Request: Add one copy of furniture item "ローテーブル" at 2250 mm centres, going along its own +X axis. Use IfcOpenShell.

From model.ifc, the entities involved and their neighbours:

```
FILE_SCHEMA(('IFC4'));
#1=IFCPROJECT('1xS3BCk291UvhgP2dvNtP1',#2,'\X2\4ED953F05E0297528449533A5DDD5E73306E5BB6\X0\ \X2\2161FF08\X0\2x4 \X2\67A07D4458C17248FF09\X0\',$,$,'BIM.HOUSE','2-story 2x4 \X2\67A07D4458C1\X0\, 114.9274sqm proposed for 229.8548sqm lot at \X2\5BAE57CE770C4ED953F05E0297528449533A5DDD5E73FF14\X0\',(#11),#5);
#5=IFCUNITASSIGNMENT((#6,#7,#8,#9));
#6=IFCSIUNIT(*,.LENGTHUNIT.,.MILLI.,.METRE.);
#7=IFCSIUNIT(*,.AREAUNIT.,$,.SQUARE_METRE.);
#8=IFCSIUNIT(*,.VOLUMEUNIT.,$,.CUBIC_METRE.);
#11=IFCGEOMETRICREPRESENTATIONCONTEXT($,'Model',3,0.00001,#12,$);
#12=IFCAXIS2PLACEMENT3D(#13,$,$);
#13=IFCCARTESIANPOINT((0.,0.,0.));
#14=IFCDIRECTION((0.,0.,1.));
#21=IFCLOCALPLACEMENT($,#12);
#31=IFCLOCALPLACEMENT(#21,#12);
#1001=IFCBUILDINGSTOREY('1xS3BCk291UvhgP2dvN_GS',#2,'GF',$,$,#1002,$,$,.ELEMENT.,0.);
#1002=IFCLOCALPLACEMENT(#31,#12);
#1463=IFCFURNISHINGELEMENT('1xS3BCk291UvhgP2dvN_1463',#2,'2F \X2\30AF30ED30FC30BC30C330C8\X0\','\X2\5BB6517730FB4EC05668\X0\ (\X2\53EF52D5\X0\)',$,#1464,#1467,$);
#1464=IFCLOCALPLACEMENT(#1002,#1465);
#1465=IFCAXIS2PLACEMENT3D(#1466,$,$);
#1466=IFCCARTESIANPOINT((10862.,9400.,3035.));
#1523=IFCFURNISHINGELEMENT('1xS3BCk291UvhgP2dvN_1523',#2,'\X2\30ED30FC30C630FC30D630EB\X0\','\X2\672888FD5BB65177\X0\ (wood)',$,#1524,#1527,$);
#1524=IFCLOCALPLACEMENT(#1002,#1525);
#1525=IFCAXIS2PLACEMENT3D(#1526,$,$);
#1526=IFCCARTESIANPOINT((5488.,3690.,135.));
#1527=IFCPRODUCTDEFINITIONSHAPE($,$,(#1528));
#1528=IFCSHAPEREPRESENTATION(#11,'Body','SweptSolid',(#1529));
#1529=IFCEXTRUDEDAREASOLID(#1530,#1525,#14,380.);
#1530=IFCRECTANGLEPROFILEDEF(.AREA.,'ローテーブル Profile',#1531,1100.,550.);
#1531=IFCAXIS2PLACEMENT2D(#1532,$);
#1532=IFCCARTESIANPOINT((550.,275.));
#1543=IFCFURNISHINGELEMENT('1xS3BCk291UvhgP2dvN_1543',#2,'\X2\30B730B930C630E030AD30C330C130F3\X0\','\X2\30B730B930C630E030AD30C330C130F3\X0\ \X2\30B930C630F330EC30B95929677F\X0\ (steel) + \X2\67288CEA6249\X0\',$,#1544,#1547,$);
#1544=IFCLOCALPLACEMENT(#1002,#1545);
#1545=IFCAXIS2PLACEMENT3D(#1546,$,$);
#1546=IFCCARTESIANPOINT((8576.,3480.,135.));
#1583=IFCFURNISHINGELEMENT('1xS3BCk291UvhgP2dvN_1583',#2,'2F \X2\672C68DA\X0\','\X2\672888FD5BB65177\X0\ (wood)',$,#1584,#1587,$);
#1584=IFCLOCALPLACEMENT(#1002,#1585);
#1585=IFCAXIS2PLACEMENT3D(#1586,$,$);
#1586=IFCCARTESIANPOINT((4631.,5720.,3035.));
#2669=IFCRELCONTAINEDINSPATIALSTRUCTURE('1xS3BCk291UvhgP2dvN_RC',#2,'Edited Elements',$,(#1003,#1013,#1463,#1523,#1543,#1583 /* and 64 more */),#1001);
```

```python
import ifcopenshell
import ifcopenshell.api.geometry
import ifcopenshell.api.root
import ifcopenshell.util.element
import ifcopenshell.util.placement

model = ifcopenshell.open("model.ifc")


def reuse_history(source, copy):
    """copy_class also copies each property set's owner history, people and application; keep the originals."""
    for rel in copy.IsDefinedBy:
        if rel.is_a("IfcRelDefinesByProperties") and (history := rel.RelatingPropertyDefinition.OwnerHistory):
            rel.RelatingPropertyDefinition.OwnerHistory = source.OwnerHistory
            ifcopenshell.util.element.remove_deep2(model, history)


source = model.by_guid("1xS3BCk291UvhgP2dvN_1523")
base = ifcopenshell.util.placement.get_local_placement(source.ObjectPlacement)
step = base[:3, 0] * 2250.0

for i in range(1, 2):
    copy = ifcopenshell.api.root.copy_class(model, product=source)
    copy.Representation = ifcopenshell.util.element.copy_deep(
        model, source.Representation, exclude=["IfcGeometricRepresentationContext", "IfcRepresentationMap"]
    )
    reuse_history(source, copy)
    matrix = base.copy()
    matrix[:3, 3] += i * step
    print("added at", matrix[:3, 3].round(3) + 0.0)
    ifcopenshell.api.geometry.edit_object_placement(model, product=copy, matrix=matrix, is_si=False)

model.write("model_updated.ifc")
```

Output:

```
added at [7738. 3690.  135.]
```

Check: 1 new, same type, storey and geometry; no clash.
